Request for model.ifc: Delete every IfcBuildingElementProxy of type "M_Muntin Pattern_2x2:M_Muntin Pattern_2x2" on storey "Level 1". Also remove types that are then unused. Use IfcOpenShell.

First a look at what the model holds.

```python
import ifcopenshell
import ifcopenshell.util.element

model = ifcopenshell.open("model.ifc")
print(model.schema)
storey = next(s for s in model.by_type("IfcBuildingStorey") if s.Name == "Level 1")
proxies = [e for e in ifcopenshell.util.element.get_decomposition(storey) if e.is_a("IfcBuildingElementProxy")]
seen = {}
for e in proxies:
    element_type = ifcopenshell.util.element.get_type(e)
    name = element_type.Name if element_type not in (None, e) else None
    seen[name] = seen.get(name, 0) + 1
for name, count in sorted(seen.items(), key=str):
    print(count, "x", name)
```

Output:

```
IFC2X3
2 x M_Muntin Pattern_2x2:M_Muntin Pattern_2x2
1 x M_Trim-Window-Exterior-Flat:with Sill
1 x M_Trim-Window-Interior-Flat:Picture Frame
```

```python
import ifcopenshell
import ifcopenshell.api.root
import ifcopenshell.util.element

model = ifcopenshell.open("model.ifc")

storey = next(s for s in model.by_type("IfcBuildingStorey") if s.Name == "Level 1")
proxies = [e for e in ifcopenshell.util.element.get_decomposition(storey) if e.is_a("IfcBuildingElementProxy")]
targets = [e for e in proxies if (t := ifcopenshell.util.element.get_type(e)) not in (None, e) and t.Name == "M_Muntin Pattern_2x2:M_Muntin Pattern_2x2"]
types = {ifcopenshell.util.element.get_type(e) for e in targets} - {None, *targets}

for e in targets:
    ifcopenshell.api.root.remove_product(model, product=e)
print(len(targets), "removed")

unused = [t for t in types if not ifcopenshell.util.element.get_types(t)]
for t in unused:
    ifcopenshell.api.root.remove_product(model, product=t)
print(len(unused), "unused types removed")

model.write("model_updated.ifc")
```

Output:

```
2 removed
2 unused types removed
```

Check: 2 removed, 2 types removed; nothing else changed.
